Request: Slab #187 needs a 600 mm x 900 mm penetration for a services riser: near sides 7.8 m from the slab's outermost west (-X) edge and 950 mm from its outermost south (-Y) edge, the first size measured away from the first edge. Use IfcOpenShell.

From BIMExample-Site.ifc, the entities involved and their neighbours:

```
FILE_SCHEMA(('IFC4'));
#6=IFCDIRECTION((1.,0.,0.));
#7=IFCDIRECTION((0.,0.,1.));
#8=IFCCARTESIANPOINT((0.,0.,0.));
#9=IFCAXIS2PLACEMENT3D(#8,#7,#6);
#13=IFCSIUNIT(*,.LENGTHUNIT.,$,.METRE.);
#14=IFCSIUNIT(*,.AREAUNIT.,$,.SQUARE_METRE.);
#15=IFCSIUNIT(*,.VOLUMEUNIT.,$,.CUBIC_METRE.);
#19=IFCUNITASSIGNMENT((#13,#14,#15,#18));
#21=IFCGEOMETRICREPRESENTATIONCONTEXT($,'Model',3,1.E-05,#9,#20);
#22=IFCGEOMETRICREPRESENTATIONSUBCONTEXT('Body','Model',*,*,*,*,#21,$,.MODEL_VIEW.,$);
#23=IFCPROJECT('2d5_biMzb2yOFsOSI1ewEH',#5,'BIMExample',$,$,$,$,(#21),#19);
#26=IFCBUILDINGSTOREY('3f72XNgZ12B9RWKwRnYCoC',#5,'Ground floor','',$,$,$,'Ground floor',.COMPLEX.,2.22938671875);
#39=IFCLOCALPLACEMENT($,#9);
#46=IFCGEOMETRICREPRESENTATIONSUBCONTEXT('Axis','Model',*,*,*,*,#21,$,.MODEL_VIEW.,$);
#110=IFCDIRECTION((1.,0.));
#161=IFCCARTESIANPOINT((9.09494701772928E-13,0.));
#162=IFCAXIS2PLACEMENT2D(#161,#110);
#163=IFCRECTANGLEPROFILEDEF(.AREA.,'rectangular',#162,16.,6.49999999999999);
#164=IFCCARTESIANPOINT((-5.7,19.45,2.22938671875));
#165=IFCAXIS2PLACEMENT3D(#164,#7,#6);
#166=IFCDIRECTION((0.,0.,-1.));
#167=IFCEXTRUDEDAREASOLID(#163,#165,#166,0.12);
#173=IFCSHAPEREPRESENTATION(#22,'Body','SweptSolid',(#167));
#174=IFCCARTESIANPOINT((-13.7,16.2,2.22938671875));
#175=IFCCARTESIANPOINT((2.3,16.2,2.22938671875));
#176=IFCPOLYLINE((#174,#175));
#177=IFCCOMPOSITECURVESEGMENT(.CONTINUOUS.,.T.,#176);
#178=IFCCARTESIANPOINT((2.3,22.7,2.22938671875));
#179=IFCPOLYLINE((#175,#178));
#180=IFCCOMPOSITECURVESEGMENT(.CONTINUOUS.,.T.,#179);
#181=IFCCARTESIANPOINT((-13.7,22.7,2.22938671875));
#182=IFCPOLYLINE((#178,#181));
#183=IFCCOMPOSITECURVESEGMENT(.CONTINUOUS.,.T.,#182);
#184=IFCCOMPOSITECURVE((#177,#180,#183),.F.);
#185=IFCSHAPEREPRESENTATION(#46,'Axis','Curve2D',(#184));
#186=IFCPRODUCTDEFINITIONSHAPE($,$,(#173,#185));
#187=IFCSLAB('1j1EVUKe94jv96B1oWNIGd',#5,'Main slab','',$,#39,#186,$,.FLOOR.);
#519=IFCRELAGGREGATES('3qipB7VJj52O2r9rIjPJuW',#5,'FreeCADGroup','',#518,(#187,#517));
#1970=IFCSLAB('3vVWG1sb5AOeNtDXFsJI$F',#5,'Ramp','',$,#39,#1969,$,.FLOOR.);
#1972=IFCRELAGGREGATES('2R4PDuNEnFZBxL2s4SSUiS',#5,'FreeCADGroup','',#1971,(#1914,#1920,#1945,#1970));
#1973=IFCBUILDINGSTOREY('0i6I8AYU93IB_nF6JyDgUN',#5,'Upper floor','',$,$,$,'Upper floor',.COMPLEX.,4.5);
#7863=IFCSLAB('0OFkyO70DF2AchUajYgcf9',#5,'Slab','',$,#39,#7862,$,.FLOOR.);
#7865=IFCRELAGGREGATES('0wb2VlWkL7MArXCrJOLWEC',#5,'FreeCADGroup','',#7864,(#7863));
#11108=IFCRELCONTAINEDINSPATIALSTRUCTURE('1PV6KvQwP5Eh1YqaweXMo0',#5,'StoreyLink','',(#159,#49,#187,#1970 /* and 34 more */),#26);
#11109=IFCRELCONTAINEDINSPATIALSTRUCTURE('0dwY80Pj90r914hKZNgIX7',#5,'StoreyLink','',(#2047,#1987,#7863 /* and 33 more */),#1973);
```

```python
import numpy as np
import ifcopenshell
import ifcopenshell.api.feature
import ifcopenshell.api.geometry
import ifcopenshell.api.root
import ifcopenshell.geom
import ifcopenshell.util.placement
import ifcopenshell.util.representation
import ifcopenshell.util.shape
import ifcopenshell.util.unit

model = ifcopenshell.open("BIMExample-Site.ifc")
unit_scale = ifcopenshell.util.unit.calculate_unit_scale(model)
settings = ifcopenshell.geom.settings()


def volume(element):
    """Net volume in cubic metres, openings subtracted."""
    shape = ifcopenshell.geom.create_shape(settings, element)
    return ifcopenshell.util.shape.get_volume(shape.geometry)


slab = model.by_guid("1j1EVUKe94jv96B1oWNIGd")
before = volume(slab)

# Extent in the slab's own axes, in metres. The edges named are its -X and -Y sides.
slab_shape = ifcopenshell.geom.create_shape(settings, slab)
vertices = ifcopenshell.util.shape.get_vertices(slab_shape.geometry)
x_min, y_min, bottom = vertices.min(axis=0)
top = vertices[:, 2].max()

opening = ifcopenshell.api.root.create_entity(model, ifc_class="IfcOpeningElement", name="Services riser opening", predefined_type="OPENING")
context = ifcopenshell.util.representation.get_context(model, "Model", "Body", "MODEL_VIEW")
width, depth = 0.6, 0.9
outline = [(0.0, 0.0), (width, 0.0), (width, depth), (0.0, depth), (0.0, 0.0)]
# Overshoot both faces by 50 mm so the cut is clean.
shape = ifcopenshell.api.geometry.add_slab_representation(
    model, context=context, depth=top - bottom + 0.1, polyline=outline
)
ifcopenshell.api.geometry.assign_representation(model, product=opening, representation=shape)

matrix = ifcopenshell.util.placement.get_local_placement(slab.ObjectPlacement)
matrix[:, 3] = matrix @ np.append(np.array([x_min + 7.8, y_min + 0.95, bottom - 0.05]) / unit_scale, 1.0)
ifcopenshell.api.geometry.edit_object_placement(model, product=opening, matrix=matrix, is_si=False)
ifcopenshell.api.feature.add_feature(model, feature=opening, element=slab)

after = volume(slab)

print(f"slab volume {before:.3f} -> {after:.3f} m3")

model.write("BIMExample-Site_v2.ifc")
```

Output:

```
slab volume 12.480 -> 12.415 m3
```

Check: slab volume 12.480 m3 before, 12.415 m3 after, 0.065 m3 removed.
